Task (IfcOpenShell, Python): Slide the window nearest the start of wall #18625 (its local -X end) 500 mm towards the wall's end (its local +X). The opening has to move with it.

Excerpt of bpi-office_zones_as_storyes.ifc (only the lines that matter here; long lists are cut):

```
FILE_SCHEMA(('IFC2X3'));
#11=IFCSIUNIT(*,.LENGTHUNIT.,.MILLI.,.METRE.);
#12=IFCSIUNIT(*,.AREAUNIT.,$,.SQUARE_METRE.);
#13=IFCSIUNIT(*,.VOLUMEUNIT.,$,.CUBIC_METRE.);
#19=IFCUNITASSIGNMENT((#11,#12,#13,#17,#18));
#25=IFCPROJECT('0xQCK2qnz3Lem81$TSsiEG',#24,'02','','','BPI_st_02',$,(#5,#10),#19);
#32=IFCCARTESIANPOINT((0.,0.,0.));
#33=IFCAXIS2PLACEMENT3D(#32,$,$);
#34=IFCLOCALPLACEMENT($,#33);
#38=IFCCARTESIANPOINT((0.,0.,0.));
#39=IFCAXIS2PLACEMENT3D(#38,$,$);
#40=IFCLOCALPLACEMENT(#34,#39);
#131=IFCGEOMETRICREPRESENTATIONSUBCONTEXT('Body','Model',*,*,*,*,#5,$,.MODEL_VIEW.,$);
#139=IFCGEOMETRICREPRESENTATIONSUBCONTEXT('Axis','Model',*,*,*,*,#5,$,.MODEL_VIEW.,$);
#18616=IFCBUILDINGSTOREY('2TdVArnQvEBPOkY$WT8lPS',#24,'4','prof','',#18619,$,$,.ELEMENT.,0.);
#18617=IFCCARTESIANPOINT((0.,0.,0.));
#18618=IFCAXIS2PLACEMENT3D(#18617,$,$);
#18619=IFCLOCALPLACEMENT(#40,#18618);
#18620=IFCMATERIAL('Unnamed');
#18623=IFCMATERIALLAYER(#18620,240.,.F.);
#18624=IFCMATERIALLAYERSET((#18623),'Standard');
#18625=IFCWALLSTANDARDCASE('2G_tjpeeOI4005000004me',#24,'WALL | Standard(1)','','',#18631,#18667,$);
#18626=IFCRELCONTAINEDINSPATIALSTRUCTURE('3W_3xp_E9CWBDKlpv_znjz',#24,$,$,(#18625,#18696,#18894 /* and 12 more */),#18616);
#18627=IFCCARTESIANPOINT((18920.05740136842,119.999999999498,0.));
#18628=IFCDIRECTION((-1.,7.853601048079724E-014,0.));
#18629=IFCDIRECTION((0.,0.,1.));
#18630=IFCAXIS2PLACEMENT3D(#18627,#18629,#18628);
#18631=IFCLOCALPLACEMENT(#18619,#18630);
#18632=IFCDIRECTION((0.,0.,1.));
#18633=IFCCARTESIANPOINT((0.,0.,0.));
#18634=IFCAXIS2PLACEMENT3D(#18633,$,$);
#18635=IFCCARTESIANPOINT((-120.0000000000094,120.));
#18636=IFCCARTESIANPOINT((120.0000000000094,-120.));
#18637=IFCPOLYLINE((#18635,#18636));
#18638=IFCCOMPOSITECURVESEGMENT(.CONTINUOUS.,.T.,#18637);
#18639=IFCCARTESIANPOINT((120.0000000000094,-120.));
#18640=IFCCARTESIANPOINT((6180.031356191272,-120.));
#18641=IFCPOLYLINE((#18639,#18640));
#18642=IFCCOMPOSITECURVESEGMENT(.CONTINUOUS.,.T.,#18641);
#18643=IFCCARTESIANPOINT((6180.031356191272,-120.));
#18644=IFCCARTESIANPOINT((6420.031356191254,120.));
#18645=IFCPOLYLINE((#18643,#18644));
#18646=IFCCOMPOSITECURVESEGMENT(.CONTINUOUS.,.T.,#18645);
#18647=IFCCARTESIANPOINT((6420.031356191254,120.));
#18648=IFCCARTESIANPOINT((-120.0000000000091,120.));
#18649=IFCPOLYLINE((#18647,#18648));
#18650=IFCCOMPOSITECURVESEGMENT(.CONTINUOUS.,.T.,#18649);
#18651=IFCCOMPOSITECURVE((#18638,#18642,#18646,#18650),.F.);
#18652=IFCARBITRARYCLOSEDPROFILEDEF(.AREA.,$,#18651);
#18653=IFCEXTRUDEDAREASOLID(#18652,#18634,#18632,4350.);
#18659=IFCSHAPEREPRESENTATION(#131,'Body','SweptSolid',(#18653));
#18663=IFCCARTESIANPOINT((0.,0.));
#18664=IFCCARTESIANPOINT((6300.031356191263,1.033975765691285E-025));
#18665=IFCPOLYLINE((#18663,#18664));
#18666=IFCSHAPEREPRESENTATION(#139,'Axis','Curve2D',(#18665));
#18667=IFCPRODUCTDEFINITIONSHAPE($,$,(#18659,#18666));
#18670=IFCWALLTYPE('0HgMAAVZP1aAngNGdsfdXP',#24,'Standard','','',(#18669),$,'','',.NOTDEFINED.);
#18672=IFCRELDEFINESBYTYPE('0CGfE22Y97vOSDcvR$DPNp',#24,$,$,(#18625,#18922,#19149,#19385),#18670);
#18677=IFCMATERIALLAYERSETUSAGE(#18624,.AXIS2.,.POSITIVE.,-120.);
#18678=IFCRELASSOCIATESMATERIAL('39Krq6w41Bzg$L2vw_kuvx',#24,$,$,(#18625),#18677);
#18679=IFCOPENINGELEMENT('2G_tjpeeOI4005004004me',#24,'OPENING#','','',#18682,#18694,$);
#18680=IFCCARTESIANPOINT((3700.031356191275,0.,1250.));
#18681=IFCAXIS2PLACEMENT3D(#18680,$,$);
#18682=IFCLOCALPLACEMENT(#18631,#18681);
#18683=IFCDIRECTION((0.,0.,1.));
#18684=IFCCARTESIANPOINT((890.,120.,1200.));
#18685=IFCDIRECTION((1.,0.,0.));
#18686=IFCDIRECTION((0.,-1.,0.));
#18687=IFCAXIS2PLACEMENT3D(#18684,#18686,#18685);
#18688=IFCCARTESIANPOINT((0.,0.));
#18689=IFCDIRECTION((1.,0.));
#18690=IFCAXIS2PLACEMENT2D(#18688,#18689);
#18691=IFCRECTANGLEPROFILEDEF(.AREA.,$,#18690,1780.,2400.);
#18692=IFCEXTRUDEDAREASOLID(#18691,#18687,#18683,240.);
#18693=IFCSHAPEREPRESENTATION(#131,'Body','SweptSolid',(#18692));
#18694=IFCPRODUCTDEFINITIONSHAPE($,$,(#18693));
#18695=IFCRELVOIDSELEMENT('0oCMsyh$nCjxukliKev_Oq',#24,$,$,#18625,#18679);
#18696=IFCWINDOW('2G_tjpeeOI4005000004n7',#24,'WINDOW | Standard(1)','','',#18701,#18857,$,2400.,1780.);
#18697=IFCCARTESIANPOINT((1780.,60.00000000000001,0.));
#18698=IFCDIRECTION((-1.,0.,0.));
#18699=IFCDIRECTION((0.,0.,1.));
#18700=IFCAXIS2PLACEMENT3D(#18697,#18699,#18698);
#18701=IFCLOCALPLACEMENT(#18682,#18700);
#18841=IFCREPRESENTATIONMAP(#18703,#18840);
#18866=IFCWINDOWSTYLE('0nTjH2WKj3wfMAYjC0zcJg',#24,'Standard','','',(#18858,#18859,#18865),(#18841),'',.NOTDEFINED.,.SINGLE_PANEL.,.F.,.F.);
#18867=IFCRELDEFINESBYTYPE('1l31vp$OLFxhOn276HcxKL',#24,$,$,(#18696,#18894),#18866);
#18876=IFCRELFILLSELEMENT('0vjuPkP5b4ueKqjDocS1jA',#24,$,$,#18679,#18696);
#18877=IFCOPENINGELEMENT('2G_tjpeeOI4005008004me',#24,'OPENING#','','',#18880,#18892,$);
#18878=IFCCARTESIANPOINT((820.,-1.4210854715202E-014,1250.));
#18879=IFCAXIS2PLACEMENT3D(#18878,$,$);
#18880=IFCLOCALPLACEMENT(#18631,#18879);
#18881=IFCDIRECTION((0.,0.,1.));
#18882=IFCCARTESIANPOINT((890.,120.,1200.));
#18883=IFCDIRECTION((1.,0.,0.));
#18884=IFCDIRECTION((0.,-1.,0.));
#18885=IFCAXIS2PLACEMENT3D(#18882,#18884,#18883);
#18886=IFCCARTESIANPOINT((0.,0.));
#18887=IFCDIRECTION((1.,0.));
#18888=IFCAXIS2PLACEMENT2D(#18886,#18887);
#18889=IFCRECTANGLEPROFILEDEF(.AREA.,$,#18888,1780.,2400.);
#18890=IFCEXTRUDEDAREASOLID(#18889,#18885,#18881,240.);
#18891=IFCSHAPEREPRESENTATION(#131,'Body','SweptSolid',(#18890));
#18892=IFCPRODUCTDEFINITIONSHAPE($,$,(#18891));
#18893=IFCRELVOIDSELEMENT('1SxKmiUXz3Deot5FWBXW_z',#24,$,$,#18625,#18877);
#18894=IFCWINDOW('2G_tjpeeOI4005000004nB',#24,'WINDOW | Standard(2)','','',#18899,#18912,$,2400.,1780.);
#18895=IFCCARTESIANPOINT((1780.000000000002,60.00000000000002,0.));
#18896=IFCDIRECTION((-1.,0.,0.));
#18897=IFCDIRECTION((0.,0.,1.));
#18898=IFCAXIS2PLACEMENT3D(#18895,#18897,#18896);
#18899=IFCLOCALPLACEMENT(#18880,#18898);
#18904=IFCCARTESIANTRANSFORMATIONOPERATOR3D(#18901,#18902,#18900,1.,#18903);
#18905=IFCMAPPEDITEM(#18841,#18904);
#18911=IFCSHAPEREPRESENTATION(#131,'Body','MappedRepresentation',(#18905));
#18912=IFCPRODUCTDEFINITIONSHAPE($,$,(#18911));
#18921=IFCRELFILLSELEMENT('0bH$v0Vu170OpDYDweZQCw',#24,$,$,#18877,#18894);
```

```python
import ifcopenshell
import ifcopenshell.api.geometry
import ifcopenshell.util.placement

model = ifcopenshell.open("bpi-office_zones_as_storyes.ifc")

window = model.by_id(18894)
opening = window.FillsVoids[0].RelatingOpeningElement
wall = opening.VoidsElements[0].RelatingBuildingElement

wall_matrix = ifcopenshell.util.placement.get_local_placement(wall.ObjectPlacement)
shift = wall_matrix[:3, 0] * 500.0
before = ifcopenshell.util.placement.get_local_placement(window.ObjectPlacement)[:3, 3].copy()

# The window is placed relative to its opening, so it follows when the opening moves.
matrix = ifcopenshell.util.placement.get_local_placement(opening.ObjectPlacement)
matrix[:3, 3] += shift
ifcopenshell.api.geometry.edit_object_placement(
    model, product=opening, matrix=matrix, is_si=False, should_transform_children=True
)

after = ifcopenshell.util.placement.get_local_placement(window.ObjectPlacement)[:3, 3]
print("window moved by", (after - before).round(3) + 0.0)

model.write("bpi-office_zones_as_storyes-out.ifc")
```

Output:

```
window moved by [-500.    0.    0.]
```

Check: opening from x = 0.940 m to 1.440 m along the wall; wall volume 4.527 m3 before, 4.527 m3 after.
